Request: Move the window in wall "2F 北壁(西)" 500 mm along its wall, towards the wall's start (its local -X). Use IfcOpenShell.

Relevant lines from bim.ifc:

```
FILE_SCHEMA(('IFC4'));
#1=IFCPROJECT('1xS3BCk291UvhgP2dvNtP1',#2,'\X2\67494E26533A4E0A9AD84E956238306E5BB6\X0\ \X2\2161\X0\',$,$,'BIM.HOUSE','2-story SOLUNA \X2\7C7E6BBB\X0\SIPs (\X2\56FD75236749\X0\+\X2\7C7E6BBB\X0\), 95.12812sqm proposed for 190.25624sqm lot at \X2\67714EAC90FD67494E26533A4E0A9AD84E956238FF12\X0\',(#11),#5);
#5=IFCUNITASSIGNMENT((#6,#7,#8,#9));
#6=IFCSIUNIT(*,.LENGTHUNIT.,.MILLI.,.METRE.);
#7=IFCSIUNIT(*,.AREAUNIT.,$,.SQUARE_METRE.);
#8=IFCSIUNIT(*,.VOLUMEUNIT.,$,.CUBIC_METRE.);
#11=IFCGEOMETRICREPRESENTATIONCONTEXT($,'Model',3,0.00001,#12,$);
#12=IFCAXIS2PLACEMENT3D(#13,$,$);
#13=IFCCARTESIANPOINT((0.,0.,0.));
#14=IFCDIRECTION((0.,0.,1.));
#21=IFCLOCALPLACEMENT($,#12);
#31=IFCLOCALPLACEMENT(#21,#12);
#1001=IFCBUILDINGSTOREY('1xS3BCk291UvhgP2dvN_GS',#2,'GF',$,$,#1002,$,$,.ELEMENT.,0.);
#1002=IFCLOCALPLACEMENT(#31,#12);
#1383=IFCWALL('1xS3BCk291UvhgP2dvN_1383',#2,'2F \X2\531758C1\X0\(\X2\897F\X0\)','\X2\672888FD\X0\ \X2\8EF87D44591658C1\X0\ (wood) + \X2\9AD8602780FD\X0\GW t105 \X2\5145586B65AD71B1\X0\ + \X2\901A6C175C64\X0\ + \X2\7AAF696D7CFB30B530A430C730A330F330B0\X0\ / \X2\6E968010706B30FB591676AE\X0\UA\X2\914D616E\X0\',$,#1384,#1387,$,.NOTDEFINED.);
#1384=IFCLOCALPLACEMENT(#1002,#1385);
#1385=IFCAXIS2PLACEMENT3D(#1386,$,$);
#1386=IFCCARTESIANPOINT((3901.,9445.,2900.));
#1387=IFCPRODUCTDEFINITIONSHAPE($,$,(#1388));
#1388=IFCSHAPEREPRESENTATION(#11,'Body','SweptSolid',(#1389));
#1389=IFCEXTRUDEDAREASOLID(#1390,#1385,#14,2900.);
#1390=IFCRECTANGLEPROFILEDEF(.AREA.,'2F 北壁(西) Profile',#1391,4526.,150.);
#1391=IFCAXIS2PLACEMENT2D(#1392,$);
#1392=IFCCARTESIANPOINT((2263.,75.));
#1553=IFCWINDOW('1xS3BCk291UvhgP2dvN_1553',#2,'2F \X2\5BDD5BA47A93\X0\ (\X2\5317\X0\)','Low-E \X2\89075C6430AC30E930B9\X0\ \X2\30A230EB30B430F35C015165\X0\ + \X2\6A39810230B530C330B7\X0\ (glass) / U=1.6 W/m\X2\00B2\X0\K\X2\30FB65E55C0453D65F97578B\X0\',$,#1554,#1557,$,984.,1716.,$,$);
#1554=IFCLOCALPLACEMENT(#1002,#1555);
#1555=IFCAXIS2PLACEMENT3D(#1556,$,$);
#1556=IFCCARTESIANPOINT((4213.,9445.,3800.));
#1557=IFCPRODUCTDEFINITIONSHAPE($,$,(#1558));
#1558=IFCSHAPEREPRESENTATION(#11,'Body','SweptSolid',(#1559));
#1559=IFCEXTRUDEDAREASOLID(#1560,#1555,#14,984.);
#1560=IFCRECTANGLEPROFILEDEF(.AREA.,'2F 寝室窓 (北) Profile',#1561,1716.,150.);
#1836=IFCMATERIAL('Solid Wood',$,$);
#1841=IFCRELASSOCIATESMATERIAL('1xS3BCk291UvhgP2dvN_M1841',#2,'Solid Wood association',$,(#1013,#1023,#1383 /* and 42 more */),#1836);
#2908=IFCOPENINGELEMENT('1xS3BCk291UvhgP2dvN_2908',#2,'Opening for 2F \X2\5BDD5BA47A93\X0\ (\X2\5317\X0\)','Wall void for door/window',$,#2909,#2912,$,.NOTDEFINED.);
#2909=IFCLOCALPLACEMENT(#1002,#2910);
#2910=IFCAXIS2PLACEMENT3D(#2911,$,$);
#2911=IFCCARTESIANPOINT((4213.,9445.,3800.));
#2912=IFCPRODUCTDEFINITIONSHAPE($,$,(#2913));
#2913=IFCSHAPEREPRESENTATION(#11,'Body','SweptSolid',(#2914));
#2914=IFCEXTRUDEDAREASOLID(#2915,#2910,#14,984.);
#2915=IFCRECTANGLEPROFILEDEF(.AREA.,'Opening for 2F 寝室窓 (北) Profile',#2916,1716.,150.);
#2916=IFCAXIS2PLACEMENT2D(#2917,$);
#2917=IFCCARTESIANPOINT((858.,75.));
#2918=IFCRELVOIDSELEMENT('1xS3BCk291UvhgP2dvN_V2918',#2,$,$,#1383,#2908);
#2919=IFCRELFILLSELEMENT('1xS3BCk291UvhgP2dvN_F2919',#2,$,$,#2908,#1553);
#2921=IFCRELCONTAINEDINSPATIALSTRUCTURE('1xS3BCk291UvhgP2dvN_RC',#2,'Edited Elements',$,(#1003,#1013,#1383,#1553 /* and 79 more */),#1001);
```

```python
import ifcopenshell
import ifcopenshell.api.geometry
import ifcopenshell.util.placement
import ifcopenshell.util.unit

model = ifcopenshell.open("bim.ifc")
unit_scale = ifcopenshell.util.unit.calculate_unit_scale(model)

window = model.by_guid("1xS3BCk291UvhgP2dvN_1553")
opening = window.FillsVoids[0].RelatingOpeningElement
wall = opening.VoidsElements[0].RelatingBuildingElement

wall_matrix = ifcopenshell.util.placement.get_local_placement(wall.ObjectPlacement)
shift = wall_matrix[:3, 0] * -0.5 / unit_scale
before = ifcopenshell.util.placement.get_local_placement(window.ObjectPlacement)[:3, 3].copy()

# The window is not placed relative to its opening, so move both.
for product in (opening, window):
    matrix = ifcopenshell.util.placement.get_local_placement(product.ObjectPlacement)
    matrix[:3, 3] += shift
    ifcopenshell.api.geometry.edit_object_placement(model, product=product, matrix=matrix, is_si=False)

after = ifcopenshell.util.placement.get_local_placement(window.ObjectPlacement)[:3, 3]
print("window moved by", (after - before).round(3) + 0.0)

model.write("bim_edited.ifc")
```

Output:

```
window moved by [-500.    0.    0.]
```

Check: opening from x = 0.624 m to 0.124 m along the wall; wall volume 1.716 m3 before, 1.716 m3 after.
